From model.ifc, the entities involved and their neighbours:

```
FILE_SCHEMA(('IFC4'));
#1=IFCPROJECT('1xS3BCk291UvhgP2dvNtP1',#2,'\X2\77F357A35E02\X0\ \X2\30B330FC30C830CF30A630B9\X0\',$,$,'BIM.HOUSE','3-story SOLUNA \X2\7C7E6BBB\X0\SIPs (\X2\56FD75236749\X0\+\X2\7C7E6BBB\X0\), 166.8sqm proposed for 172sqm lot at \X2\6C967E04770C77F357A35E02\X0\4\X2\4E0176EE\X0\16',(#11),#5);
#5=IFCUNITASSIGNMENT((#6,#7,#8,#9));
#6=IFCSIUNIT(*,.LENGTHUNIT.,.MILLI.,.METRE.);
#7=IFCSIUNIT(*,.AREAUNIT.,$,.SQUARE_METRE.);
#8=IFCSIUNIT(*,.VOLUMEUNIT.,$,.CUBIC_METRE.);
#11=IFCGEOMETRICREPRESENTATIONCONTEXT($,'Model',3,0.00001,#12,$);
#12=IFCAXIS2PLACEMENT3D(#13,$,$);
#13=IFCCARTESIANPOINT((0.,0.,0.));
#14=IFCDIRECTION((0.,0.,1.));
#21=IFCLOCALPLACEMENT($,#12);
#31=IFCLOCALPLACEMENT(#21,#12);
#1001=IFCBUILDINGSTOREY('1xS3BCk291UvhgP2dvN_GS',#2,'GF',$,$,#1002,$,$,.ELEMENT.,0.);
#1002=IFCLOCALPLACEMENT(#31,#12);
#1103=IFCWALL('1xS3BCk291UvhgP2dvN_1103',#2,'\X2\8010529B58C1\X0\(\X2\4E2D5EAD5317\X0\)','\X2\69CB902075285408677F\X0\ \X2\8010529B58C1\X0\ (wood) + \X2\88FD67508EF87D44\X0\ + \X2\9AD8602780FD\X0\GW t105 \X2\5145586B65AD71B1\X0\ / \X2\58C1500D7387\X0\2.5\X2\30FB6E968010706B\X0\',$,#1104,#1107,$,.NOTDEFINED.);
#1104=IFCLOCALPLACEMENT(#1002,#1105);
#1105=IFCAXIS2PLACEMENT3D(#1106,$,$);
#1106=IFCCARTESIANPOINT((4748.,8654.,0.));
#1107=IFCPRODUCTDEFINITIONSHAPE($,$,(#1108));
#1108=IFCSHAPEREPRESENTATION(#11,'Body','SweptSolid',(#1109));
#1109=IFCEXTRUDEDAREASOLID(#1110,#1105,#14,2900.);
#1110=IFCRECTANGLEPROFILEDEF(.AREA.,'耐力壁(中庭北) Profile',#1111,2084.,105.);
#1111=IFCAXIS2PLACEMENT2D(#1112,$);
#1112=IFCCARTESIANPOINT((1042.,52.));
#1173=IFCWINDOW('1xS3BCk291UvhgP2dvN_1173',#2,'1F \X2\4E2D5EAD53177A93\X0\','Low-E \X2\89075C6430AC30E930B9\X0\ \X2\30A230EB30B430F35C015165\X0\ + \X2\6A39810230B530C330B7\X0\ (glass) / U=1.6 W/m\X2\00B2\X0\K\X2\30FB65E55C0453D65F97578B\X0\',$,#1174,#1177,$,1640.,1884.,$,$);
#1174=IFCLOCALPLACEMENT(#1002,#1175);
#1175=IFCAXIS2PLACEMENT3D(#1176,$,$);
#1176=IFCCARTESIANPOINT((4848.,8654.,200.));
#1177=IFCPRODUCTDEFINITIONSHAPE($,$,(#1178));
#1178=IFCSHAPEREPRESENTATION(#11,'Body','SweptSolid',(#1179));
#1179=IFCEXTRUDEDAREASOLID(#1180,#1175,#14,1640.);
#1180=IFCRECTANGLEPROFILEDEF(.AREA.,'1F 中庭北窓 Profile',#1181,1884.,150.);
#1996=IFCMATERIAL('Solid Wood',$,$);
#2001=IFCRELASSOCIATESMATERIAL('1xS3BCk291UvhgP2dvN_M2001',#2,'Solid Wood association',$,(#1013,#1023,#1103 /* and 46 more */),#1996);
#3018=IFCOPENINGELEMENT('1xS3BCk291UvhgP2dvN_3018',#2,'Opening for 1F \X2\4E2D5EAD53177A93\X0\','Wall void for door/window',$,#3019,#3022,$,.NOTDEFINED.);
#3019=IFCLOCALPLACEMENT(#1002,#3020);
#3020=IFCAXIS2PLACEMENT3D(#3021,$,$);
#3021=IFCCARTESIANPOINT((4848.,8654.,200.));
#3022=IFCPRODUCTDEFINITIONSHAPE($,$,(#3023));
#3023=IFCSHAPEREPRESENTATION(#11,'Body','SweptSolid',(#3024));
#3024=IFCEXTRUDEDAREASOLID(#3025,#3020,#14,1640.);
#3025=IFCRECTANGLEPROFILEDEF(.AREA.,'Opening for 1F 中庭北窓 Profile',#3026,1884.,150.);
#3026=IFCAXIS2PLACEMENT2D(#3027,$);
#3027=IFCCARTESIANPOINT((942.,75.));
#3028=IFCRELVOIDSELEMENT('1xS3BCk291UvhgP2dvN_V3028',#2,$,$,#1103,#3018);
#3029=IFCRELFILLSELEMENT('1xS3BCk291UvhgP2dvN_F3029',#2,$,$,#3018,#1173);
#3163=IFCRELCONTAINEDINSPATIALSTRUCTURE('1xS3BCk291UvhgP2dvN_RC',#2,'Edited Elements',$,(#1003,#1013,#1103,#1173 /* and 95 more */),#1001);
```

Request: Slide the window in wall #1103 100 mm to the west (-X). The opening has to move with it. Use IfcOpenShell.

```python
import ifcopenshell
import ifcopenshell.api.geometry
import ifcopenshell.util.placement
import ifcopenshell.util.unit

model = ifcopenshell.open("model.ifc")
unit_scale = ifcopenshell.util.unit.calculate_unit_scale(model)

window = model.by_guid("1xS3BCk291UvhgP2dvN_1173")
opening = window.FillsVoids[0].RelatingOpeningElement
wall = opening.VoidsElements[0].RelatingBuildingElement

wall_matrix = ifcopenshell.util.placement.get_local_placement(wall.ObjectPlacement)
shift = wall_matrix[:3, 0] * -0.1 / unit_scale
before = ifcopenshell.util.placement.get_local_placement(window.ObjectPlacement)[:3, 3].copy()

# The window is not placed relative to its opening, so move both.
for product in (opening, window):
    matrix = ifcopenshell.util.placement.get_local_placement(product.ObjectPlacement)
    matrix[:3, 3] += shift
    ifcopenshell.api.geometry.edit_object_placement(model, product=product, matrix=matrix, is_si=False)

after = ifcopenshell.util.placement.get_local_placement(window.ObjectPlacement)[:3, 3]
print("window moved by", (after - before).round(3) + 0.0)

model.write("model_updated.ifc")
```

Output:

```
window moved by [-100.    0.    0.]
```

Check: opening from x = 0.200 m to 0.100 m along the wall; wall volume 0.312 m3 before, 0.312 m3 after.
